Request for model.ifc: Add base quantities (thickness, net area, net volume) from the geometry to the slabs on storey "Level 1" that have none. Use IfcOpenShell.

First a look at what the model holds.

```python
import ifcopenshell
import ifcopenshell.util.element
import ifcopenshell.util.unit

model = ifcopenshell.open("model.ifc")
print(model.schema)
for unit_type in ("LENGTHUNIT", "AREAUNIT", "VOLUMEUNIT"):
    print(unit_type, ifcopenshell.util.unit.calculate_unit_scale(model, unit_type))
storey = next(s for s in model.by_type("IfcBuildingStorey") if s.Name == "Level 1")
slabs = [e for e in ifcopenshell.util.element.get_decomposition(storey) if e.is_a("IfcSlab")]
for e in sorted(slabs, key=lambda e: e.id()):
    print(e.id(), e.is_a(), e.Name, list(ifcopenshell.util.element.get_psets(e, qtos_only=True)), sep=" | ")
```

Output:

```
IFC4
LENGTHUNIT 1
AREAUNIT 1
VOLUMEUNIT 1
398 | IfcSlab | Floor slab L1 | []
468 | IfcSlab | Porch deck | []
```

```python
import ifcopenshell
import ifcopenshell.api.pset
import ifcopenshell.geom
import ifcopenshell.util.element
import ifcopenshell.util.shape
import ifcopenshell.util.unit

model = ifcopenshell.open("model.ifc")
unit_scale = ifcopenshell.util.unit.calculate_unit_scale(model)
area_scale = ifcopenshell.util.unit.calculate_unit_scale(model, "AREAUNIT")
volume_scale = ifcopenshell.util.unit.calculate_unit_scale(model, "VOLUMEUNIT")
settings = ifcopenshell.geom.settings()

storey = next(s for s in model.by_type("IfcBuildingStorey") if s.Name == "Level 1")
slabs = [e for e in ifcopenshell.util.element.get_decomposition(storey) if e.is_a("IfcSlab")]

for e in sorted(slabs, key=lambda e: e.id()):
    if ifcopenshell.util.element.get_psets(e, qtos_only=True, should_inherit=False):
        continue
    # Geometry comes back in metres, in the element's own axes.
    shape = ifcopenshell.geom.create_shape(settings, e)
    values = {
        "Width": ifcopenshell.util.shape.get_z(shape.geometry) / unit_scale,
        "NetArea": ifcopenshell.util.shape.get_footprint_area(shape.geometry) / area_scale,
        "NetVolume": ifcopenshell.util.shape.get_volume(shape.geometry) / volume_scale,
    }
    qto = ifcopenshell.api.pset.add_qto(model, product=e, name="Qto_SlabBaseQuantities")
    ifcopenshell.api.pset.edit_qto(model, qto=qto, properties=values)
    print(e.id(), {k: round(v, 3) for k, v in values.items()})

model.write("model_updated.ifc")
```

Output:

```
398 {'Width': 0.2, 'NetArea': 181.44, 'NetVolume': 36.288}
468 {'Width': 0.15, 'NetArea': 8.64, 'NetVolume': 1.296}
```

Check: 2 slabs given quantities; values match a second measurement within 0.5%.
